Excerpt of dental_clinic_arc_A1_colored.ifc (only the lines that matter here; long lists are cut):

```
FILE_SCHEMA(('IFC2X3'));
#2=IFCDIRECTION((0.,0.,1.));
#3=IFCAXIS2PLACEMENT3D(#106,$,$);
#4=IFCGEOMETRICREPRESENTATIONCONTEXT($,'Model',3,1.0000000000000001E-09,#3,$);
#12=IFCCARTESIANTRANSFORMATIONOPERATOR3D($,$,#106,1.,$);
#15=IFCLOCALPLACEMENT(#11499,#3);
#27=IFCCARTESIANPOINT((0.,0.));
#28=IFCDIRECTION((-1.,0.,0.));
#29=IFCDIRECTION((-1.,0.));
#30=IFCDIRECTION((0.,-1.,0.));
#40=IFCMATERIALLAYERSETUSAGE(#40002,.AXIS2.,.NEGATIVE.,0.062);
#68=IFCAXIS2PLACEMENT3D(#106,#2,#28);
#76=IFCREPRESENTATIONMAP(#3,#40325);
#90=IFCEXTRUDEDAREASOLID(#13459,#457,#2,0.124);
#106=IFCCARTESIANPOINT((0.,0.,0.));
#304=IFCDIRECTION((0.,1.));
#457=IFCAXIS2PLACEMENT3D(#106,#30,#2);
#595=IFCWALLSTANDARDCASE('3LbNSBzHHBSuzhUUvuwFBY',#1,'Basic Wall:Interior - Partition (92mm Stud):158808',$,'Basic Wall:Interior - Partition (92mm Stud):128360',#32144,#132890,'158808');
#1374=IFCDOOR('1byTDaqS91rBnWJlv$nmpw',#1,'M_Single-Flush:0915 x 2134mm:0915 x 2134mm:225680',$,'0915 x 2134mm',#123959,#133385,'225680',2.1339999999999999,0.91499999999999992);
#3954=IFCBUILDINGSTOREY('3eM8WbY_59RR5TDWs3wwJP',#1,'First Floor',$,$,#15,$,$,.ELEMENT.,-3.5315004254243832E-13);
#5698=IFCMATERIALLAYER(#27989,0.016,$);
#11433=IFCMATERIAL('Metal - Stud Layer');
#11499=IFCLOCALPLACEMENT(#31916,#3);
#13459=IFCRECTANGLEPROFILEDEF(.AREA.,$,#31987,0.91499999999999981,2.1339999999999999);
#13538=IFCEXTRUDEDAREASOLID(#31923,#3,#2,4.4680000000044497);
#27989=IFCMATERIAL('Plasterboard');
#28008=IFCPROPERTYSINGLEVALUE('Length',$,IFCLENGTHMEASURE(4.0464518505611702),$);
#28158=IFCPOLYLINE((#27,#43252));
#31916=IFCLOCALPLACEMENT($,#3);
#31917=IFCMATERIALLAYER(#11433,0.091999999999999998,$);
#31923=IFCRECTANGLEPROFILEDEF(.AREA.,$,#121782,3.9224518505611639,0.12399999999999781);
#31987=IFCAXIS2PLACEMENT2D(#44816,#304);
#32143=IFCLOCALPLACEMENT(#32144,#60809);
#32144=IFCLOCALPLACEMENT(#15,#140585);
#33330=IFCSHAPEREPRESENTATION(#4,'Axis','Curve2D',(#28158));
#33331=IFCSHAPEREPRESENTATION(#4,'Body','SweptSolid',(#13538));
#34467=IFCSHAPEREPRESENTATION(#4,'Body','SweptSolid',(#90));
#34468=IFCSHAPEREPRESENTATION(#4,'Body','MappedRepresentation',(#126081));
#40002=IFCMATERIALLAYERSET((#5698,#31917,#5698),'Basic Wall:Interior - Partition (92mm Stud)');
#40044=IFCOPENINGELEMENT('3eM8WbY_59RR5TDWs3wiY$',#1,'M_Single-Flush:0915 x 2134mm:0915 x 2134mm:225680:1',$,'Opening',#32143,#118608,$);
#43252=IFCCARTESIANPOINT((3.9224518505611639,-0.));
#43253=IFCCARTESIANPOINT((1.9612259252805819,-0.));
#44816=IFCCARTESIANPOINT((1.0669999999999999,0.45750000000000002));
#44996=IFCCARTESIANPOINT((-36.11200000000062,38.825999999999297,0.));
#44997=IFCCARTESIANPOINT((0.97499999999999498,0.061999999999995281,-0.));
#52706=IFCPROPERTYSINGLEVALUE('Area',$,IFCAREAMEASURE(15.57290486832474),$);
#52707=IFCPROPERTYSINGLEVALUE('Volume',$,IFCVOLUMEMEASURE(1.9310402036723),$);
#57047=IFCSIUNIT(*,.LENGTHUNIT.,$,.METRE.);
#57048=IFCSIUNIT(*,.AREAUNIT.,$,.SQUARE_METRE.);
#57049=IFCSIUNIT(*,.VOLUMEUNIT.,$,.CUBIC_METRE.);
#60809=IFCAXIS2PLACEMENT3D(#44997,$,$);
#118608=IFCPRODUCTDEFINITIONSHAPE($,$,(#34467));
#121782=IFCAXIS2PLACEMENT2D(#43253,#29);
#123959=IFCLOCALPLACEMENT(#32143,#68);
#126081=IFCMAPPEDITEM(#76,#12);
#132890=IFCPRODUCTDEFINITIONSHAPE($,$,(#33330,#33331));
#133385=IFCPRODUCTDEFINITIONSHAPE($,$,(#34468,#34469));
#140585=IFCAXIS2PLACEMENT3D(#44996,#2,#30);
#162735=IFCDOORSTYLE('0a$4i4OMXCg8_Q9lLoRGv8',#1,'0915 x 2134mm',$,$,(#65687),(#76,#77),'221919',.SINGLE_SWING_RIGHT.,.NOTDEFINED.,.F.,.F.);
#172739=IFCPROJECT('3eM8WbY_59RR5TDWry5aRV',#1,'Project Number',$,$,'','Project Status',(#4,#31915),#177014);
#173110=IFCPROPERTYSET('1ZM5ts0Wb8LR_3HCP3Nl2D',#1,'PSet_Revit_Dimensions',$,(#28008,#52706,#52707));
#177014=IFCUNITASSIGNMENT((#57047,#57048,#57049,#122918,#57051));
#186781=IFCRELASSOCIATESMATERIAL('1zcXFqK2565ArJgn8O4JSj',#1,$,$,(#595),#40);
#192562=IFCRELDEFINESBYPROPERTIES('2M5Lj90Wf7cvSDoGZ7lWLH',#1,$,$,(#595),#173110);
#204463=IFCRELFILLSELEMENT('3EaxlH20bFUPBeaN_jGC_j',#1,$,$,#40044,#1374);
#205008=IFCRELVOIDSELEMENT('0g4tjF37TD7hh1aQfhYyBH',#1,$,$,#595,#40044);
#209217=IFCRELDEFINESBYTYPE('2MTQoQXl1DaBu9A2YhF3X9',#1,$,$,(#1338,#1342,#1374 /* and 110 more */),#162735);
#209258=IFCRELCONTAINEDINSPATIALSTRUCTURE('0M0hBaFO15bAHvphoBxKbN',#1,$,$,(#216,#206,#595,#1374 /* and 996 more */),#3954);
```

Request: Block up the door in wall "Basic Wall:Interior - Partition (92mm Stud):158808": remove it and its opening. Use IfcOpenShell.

```python
import ifcopenshell
import ifcopenshell.api.feature
import ifcopenshell.api.pset
import ifcopenshell.api.root
import ifcopenshell.geom
import ifcopenshell.util.element
import ifcopenshell.util.shape
import ifcopenshell.util.unit

model = ifcopenshell.open("dental_clinic_arc_A1_colored.ifc")
area_scale = ifcopenshell.util.unit.calculate_unit_scale(model, "AREAUNIT")
volume_scale = ifcopenshell.util.unit.calculate_unit_scale(model, "VOLUMEUNIT")
settings = ifcopenshell.geom.settings()


def volume(element):
    """Net volume in cubic metres, openings subtracted."""
    shape = ifcopenshell.geom.create_shape(settings, element)
    return ifcopenshell.util.shape.get_volume(shape.geometry)


door = model.by_guid("1byTDaqS91rBnWJlv$nmpw")
opening = door.FillsVoids[0].RelatingOpeningElement
wall = opening.VoidsElements[0].RelatingBuildingElement
before = volume(wall)

ifcopenshell.api.root.remove_product(model, product=door)
ifcopenshell.api.feature.remove_feature(model, feature=opening)

after = volume(wall)
thickness = 0.124  # wall thickness in metres

# Update the wall's stored quantities.
pset = model.by_id(ifcopenshell.util.element.get_pset(wall, "PSet_Revit_Dimensions", should_inherit=False)["id"])
ifcopenshell.api.pset.edit_pset(model, pset=pset, properties={
    "Area": model.create_entity("IfcAreaMeasure", after / thickness / area_scale),
    "Volume": model.create_entity("IfcVolumeMeasure", after / volume_scale),
})

print(f"wall volume {before:.3f} -> {after:.3f} m3")

model.write("dental_clinic_arc_A1_colored_v2.ifc")
```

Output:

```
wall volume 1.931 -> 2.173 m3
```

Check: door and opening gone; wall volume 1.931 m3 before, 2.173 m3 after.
